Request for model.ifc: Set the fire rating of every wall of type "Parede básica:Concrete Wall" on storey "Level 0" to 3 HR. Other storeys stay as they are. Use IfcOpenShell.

First a look at what the model holds.

```python
import ifcopenshell
import ifcopenshell.util.element

model = ifcopenshell.open("model.ifc")
print(model.schema)
storey = next(s for s in model.by_type("IfcBuildingStorey") if s.Name == "Level 0")
walls = [e for e in ifcopenshell.util.element.get_decomposition(storey) if e.is_a("IfcWall")]
seen = {}
for e in walls:
    element_type = ifcopenshell.util.element.get_type(e)
    key = (element_type.Name if element_type != e and element_type else None, ifcopenshell.util.element.get_pset(e, "Pset_WallCommon", "FireRating"))
    seen[key] = seen.get(key, 0) + 1
for (name, value), count in sorted(seen.items(), key=str):
    print(count, "x", name, "|", value)
```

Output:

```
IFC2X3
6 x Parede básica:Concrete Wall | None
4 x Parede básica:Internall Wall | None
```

```python
import ifcopenshell
import ifcopenshell.api.pset
import ifcopenshell.util.element

model = ifcopenshell.open("model.ifc")

storey = next(s for s in model.by_type("IfcBuildingStorey") if s.Name == "Level 0")
walls = [e for e in ifcopenshell.util.element.get_decomposition(storey) if e.is_a("IfcWall")]

count = 0
for e in walls:
    element_type = ifcopenshell.util.element.get_type(e)
    if element_type in (None, e) or element_type.Name != "Parede básica:Concrete Wall":
        continue
    # add_pset returns the element's existing set when there is one.
    pset = ifcopenshell.api.pset.add_pset(model, product=e, name="Pset_WallCommon")
    ifcopenshell.api.pset.edit_pset(model, pset=pset, properties={"FireRating": "3 HR"})
    count += 1

print(count, "walls updated")

model.write("model_edited.ifc")
```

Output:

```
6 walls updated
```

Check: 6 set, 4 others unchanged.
